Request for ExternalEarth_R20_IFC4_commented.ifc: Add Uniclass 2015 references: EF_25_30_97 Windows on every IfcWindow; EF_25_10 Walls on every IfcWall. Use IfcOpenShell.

First a look at what the model holds.

```python
import ifcopenshell

model = ifcopenshell.open("ExternalEarth_R20_IFC4_commented.ifc")
print(model.schema)
print("classifications:", [c.Name for c in model.by_type("IfcClassification")])
for ifc_class in ("IfcDoor", "IfcRoof", "IfcStair", "IfcWall", "IfcWindow"):
    print(ifc_class, len(model.by_type(ifc_class)))
```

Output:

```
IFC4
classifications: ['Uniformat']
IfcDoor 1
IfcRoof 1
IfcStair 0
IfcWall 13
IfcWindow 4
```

```python
import ifcopenshell
import ifcopenshell.api.classification

model = ifcopenshell.open("ExternalEarth_R20_IFC4_commented.ifc")

system = ifcopenshell.api.classification.add_classification(model, classification="Uniclass 2015")

codes = {
    "IfcWindow": ("EF_25_30_97", "Windows"),
    "IfcWall": ("EF_25_10", "Walls"),
}
for ifc_class, (code, name) in codes.items():
    products = model.by_type(ifc_class)
    ifcopenshell.api.classification.add_reference(
        model, products=products, classification=system, identification=code, name=name
    )
    print(code, len(products))

model.write("ExternalEarth_R20_IFC4_commented-out.ifc")
```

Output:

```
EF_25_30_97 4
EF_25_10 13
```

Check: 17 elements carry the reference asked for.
